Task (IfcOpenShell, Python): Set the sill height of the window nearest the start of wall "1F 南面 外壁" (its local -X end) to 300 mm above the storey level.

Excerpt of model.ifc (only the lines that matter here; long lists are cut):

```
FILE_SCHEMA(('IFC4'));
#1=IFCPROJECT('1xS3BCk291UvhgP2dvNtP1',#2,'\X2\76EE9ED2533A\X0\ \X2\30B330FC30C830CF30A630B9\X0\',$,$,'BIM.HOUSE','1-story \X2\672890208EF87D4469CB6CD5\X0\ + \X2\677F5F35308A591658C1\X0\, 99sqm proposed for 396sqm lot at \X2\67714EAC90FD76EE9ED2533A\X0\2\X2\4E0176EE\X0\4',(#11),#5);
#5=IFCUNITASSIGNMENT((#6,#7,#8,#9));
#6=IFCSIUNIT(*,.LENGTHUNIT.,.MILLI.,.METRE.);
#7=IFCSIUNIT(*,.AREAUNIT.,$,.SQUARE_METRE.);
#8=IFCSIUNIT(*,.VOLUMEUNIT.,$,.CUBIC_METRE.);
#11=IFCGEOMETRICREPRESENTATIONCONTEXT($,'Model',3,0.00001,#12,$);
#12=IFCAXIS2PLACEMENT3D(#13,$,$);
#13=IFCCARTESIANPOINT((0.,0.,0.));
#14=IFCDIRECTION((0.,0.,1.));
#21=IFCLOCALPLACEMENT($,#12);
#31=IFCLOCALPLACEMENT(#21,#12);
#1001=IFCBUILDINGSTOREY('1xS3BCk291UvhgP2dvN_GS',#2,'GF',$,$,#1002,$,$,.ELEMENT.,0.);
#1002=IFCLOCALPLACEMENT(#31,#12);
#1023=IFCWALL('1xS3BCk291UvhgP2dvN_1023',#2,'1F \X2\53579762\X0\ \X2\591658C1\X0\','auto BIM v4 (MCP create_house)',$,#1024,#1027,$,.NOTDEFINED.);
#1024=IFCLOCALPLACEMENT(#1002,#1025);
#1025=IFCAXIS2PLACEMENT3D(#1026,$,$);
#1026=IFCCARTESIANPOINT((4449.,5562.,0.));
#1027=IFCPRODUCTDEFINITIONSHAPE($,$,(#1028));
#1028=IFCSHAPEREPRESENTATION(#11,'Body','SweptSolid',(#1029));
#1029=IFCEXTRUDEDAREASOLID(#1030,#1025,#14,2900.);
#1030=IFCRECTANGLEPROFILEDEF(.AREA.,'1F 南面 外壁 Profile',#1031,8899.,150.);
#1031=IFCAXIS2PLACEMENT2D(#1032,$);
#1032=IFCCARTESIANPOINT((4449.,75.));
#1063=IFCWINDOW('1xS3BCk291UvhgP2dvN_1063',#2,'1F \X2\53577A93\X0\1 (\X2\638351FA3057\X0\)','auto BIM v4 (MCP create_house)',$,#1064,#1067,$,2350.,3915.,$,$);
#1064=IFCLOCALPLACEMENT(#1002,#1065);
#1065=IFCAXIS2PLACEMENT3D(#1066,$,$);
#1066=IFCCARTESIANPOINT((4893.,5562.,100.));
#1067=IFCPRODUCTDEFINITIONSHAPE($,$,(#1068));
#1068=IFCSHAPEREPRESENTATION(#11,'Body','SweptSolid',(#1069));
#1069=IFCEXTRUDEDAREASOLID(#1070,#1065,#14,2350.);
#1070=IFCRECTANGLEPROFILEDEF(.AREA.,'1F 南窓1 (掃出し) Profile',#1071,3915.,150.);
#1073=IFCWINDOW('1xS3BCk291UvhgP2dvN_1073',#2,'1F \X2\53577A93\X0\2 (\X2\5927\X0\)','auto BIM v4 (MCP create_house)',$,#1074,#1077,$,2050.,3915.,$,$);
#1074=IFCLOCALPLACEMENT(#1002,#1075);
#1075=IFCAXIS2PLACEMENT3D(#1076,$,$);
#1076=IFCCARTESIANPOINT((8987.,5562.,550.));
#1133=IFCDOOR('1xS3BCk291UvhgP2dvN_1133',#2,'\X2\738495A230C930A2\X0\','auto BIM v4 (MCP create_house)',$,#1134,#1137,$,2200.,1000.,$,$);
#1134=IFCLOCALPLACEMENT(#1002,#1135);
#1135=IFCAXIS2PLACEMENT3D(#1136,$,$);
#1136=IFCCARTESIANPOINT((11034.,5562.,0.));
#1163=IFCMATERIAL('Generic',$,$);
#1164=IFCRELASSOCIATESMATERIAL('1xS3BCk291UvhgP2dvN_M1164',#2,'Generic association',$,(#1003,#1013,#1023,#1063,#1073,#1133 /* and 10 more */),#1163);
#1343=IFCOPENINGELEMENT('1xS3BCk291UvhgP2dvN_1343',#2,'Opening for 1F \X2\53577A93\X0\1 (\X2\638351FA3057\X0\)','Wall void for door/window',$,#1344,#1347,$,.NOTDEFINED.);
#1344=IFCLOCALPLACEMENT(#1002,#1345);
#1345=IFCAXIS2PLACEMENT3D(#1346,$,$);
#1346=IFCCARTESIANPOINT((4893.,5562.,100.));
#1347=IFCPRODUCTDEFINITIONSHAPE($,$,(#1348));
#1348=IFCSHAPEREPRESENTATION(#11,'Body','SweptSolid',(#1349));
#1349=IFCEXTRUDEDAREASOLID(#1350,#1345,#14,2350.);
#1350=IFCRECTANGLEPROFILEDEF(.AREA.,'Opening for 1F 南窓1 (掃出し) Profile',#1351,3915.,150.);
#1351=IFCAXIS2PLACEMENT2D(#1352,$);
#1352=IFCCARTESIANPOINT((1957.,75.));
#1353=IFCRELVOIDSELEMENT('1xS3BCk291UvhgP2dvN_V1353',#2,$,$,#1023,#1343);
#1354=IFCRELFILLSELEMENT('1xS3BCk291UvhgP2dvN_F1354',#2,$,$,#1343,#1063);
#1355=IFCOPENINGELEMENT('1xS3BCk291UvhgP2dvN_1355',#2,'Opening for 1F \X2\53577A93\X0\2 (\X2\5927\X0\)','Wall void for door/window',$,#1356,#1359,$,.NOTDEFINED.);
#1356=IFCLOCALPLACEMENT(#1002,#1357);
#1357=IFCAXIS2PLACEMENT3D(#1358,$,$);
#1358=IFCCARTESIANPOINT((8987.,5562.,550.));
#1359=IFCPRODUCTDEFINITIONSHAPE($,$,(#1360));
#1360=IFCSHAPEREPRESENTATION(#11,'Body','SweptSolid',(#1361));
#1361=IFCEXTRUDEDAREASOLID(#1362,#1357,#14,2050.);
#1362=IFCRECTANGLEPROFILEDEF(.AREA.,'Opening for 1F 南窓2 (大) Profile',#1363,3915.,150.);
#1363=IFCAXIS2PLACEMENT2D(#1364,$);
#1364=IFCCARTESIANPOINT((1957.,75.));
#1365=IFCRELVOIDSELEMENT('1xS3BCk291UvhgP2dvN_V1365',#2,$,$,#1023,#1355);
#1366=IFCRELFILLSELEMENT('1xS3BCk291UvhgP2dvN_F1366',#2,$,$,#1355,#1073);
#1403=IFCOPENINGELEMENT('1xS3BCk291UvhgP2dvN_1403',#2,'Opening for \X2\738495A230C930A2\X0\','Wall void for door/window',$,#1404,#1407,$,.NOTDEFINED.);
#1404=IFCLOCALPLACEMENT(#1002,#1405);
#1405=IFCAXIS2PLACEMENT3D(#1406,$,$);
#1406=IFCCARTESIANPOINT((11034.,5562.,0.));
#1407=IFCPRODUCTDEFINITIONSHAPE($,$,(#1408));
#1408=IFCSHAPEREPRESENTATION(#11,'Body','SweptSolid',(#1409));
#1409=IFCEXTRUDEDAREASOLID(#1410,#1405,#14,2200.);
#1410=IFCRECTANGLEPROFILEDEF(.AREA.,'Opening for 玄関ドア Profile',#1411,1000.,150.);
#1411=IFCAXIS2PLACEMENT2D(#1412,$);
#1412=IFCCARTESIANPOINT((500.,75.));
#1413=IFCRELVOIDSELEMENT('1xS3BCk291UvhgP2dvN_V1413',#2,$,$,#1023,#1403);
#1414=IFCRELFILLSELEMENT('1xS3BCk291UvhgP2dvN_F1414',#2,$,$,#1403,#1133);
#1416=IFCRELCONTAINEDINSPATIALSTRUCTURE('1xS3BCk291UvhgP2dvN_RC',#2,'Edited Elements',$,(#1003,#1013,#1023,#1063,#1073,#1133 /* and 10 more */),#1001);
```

```python
import numpy as np
import ifcopenshell
import ifcopenshell.api.geometry
import ifcopenshell.geom
import ifcopenshell.util.element
import ifcopenshell.util.placement
import ifcopenshell.util.shape
import ifcopenshell.util.unit

model = ifcopenshell.open("model.ifc")
unit_scale = ifcopenshell.util.unit.calculate_unit_scale(model)

window = model.by_id(1063)
opening = window.FillsVoids[0].RelatingOpeningElement
storey = ifcopenshell.util.element.get_container(window, ifc_class="IfcBuildingStorey")
level = ifcopenshell.util.placement.get_local_placement(storey.ObjectPlacement)[2, 3]

# The opening's origin need not be at the sill, so measure its lowest point.
shape = ifcopenshell.geom.create_shape(ifcopenshell.geom.settings(), opening)
bottom = ifcopenshell.util.shape.get_shape_bottom_elevation(shape, shape.geometry) / unit_scale
dz = level + 0.3 / unit_scale - bottom

shift = np.array([0.0, 0.0, dz])
# The window is not placed relative to its opening, so move both.
for product in (opening, window):
    matrix = ifcopenshell.util.placement.get_local_placement(product.ObjectPlacement)
    matrix[:3, 3] += shift
    ifcopenshell.api.geometry.edit_object_placement(model, product=product, matrix=matrix, is_si=False)

print(f"moved by {dz * unit_scale:+.3f} m")

model.write("model_updated.ifc")
```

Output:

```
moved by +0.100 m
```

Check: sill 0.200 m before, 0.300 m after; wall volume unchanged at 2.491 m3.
